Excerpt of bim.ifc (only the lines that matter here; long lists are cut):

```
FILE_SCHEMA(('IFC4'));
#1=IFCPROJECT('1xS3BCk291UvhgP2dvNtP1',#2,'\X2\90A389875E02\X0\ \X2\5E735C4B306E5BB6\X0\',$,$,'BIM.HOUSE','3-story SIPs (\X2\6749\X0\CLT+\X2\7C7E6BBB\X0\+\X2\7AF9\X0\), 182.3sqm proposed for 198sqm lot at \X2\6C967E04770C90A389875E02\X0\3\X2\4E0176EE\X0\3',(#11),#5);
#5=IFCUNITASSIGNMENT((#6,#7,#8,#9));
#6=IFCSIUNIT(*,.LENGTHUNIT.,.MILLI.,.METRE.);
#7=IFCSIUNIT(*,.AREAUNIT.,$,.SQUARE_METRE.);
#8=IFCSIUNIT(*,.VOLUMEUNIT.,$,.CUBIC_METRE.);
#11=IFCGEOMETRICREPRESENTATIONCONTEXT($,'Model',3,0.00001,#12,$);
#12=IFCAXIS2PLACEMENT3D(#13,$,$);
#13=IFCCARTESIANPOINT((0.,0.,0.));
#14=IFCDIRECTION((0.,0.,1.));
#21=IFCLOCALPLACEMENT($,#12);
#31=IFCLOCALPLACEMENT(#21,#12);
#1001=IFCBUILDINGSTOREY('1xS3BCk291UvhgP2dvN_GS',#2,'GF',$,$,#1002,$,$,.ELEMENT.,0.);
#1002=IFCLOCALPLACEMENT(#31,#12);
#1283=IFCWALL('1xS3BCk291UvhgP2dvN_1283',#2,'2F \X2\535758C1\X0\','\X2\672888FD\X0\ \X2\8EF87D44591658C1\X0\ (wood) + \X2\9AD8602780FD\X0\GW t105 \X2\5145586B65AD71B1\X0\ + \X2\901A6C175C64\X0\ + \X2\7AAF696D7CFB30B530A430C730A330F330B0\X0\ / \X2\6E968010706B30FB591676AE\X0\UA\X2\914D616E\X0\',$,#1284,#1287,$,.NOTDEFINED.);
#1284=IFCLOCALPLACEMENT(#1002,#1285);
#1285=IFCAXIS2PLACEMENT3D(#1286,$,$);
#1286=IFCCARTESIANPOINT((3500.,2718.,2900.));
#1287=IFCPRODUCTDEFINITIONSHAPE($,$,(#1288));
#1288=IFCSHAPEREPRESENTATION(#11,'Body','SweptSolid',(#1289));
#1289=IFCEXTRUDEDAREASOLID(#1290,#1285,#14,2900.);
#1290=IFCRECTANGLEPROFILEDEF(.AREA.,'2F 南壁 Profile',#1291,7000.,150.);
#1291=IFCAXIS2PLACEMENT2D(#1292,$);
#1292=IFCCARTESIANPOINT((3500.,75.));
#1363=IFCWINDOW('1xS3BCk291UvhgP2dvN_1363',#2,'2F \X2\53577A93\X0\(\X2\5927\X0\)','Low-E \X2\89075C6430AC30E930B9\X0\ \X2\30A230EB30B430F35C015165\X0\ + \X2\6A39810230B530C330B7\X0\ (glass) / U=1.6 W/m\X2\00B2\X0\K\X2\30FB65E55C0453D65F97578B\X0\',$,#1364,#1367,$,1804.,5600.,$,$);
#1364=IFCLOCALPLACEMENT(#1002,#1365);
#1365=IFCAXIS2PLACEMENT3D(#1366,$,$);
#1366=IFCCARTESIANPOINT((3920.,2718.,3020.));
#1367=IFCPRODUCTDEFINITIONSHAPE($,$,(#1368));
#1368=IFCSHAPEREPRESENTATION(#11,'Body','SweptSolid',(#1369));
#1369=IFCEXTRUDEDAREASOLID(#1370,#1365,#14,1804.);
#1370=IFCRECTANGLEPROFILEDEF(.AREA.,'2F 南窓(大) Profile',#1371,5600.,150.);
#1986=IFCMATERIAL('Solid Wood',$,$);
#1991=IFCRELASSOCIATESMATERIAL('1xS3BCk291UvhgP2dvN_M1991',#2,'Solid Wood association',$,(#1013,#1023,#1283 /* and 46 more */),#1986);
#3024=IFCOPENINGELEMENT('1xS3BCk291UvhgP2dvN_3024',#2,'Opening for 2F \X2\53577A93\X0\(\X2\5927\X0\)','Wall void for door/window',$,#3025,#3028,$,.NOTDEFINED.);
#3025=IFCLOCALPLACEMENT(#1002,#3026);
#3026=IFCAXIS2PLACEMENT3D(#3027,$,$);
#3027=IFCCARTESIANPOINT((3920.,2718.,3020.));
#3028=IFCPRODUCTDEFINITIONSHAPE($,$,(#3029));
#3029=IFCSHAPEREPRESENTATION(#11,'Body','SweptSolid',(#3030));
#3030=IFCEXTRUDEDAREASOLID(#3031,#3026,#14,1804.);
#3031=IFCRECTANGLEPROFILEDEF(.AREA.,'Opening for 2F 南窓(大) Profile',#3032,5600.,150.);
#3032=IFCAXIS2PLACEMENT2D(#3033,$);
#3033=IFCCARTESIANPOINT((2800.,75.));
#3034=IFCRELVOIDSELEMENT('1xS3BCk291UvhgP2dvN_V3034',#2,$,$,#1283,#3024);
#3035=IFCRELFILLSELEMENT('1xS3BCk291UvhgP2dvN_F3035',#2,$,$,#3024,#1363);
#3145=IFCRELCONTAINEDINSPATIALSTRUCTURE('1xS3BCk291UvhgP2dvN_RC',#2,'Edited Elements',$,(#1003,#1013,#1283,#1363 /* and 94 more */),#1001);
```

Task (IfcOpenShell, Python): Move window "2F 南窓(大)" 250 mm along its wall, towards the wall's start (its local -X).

```python
import ifcopenshell
import ifcopenshell.api.geometry
import ifcopenshell.util.placement

model = ifcopenshell.open("bim.ifc")

window = model.by_guid("1xS3BCk291UvhgP2dvN_1363")
opening = window.FillsVoids[0].RelatingOpeningElement
wall = opening.VoidsElements[0].RelatingBuildingElement

wall_matrix = ifcopenshell.util.placement.get_local_placement(wall.ObjectPlacement)
shift = wall_matrix[:3, 0] * -250.0
before = ifcopenshell.util.placement.get_local_placement(window.ObjectPlacement)[:3, 3].copy()

# The window is not placed relative to its opening, so move both.
for product in (opening, window):
    matrix = ifcopenshell.util.placement.get_local_placement(product.ObjectPlacement)
    matrix[:3, 3] += shift
    ifcopenshell.api.geometry.edit_object_placement(model, product=product, matrix=matrix, is_si=False)

after = ifcopenshell.util.placement.get_local_placement(window.ObjectPlacement)[:3, 3]
print("window moved by", (after - before).round(3) + 0.0)

model.write("bim-out.ifc")
```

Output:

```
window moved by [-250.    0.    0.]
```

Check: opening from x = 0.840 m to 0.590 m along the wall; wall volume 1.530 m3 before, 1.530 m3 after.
